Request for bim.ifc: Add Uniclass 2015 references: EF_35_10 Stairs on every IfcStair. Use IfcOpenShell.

First a look at what the model holds.

```python
import ifcopenshell

model = ifcopenshell.open("bim.ifc")
print(model.schema)
print("classifications:", [c.Name for c in model.by_type("IfcClassification")])
for ifc_class in ("IfcDoor", "IfcRoof", "IfcStair", "IfcWall", "IfcWindow"):
    print(ifc_class, len(model.by_type(ifc_class)))
```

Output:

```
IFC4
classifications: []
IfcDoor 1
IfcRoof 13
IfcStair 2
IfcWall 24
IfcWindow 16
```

```python
import ifcopenshell
import ifcopenshell.api.classification

model = ifcopenshell.open("bim.ifc")

system = ifcopenshell.api.classification.add_classification(model, classification="Uniclass 2015")

codes = {
    "IfcStair": ("EF_35_10", "Stairs"),
}
for ifc_class, (code, name) in codes.items():
    products = model.by_type(ifc_class)
    ifcopenshell.api.classification.add_reference(
        model, products=products, classification=system, identification=code, name=name
    )
    print(code, len(products))

model.write("bim_edited.ifc")
```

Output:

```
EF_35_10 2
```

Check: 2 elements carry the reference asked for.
